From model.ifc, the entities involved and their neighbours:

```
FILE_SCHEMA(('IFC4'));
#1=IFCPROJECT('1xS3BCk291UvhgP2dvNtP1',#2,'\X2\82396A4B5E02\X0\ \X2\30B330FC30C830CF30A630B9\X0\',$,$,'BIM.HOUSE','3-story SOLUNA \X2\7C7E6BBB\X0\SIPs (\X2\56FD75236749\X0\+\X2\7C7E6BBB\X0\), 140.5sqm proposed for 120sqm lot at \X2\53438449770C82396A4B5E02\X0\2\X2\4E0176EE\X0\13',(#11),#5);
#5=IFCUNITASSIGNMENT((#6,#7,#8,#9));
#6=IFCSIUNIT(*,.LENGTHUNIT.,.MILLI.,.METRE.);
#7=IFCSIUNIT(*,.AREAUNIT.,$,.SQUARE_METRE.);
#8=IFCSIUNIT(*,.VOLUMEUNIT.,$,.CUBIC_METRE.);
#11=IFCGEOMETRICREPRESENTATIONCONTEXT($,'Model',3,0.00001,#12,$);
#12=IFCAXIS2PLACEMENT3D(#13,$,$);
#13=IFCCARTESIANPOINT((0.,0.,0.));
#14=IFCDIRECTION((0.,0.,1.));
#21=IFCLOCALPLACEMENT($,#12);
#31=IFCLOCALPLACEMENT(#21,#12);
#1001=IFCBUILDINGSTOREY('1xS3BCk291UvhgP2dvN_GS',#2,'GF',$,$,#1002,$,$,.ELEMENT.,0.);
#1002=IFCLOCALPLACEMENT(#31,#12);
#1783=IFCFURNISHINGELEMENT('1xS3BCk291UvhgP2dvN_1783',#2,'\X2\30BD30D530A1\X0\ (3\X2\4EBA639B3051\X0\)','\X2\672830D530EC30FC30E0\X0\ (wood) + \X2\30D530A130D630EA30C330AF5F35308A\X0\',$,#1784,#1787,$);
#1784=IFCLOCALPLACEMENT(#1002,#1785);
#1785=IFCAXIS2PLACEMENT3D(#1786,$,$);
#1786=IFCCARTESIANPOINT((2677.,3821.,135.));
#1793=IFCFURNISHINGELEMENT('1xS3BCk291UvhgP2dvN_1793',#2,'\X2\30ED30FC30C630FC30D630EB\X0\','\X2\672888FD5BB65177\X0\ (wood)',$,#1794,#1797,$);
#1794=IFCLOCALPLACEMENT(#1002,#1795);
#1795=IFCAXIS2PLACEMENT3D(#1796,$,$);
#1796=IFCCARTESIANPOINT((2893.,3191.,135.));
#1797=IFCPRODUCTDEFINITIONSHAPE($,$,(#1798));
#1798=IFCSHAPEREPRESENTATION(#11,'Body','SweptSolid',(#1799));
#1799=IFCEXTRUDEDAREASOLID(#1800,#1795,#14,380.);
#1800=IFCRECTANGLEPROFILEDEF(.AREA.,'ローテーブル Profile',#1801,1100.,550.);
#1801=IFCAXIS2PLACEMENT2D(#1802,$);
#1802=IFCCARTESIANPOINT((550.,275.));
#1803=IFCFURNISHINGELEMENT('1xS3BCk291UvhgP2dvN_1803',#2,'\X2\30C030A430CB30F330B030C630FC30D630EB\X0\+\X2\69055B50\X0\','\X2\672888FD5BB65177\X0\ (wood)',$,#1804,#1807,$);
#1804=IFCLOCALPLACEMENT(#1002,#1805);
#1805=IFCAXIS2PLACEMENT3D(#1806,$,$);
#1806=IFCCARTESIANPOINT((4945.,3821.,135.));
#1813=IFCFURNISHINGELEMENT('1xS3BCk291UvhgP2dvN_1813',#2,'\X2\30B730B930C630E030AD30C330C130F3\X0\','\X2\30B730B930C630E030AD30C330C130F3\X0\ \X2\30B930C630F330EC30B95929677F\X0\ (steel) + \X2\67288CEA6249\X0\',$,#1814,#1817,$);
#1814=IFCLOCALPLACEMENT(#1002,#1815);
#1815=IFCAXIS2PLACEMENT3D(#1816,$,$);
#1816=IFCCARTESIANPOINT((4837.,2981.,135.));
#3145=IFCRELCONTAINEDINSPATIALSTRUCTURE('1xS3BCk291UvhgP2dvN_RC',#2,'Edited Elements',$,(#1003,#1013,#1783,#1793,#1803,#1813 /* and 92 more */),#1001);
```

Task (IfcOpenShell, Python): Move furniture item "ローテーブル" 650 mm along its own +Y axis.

```python
import ifcopenshell
import ifcopenshell.api.geometry
import ifcopenshell.util.placement
import ifcopenshell.util.unit

model = ifcopenshell.open("model.ifc")
unit_scale = ifcopenshell.util.unit.calculate_unit_scale(model)

item = model.by_guid("1xS3BCk291UvhgP2dvN_1793")
matrix = ifcopenshell.util.placement.get_local_placement(item.ObjectPlacement)
matrix[:3, 3] += matrix[:3, 1] * 0.65 / unit_scale
ifcopenshell.api.geometry.edit_object_placement(model, product=item, matrix=matrix, is_si=False)

print(ifcopenshell.util.placement.get_local_placement(item.ObjectPlacement).round(3) + 0.0)

model.write("model_edited.ifc")
```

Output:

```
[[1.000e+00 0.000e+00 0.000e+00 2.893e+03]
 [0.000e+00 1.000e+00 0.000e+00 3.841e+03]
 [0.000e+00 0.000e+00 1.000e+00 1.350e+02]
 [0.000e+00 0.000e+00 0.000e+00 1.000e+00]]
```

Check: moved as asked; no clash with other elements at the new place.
